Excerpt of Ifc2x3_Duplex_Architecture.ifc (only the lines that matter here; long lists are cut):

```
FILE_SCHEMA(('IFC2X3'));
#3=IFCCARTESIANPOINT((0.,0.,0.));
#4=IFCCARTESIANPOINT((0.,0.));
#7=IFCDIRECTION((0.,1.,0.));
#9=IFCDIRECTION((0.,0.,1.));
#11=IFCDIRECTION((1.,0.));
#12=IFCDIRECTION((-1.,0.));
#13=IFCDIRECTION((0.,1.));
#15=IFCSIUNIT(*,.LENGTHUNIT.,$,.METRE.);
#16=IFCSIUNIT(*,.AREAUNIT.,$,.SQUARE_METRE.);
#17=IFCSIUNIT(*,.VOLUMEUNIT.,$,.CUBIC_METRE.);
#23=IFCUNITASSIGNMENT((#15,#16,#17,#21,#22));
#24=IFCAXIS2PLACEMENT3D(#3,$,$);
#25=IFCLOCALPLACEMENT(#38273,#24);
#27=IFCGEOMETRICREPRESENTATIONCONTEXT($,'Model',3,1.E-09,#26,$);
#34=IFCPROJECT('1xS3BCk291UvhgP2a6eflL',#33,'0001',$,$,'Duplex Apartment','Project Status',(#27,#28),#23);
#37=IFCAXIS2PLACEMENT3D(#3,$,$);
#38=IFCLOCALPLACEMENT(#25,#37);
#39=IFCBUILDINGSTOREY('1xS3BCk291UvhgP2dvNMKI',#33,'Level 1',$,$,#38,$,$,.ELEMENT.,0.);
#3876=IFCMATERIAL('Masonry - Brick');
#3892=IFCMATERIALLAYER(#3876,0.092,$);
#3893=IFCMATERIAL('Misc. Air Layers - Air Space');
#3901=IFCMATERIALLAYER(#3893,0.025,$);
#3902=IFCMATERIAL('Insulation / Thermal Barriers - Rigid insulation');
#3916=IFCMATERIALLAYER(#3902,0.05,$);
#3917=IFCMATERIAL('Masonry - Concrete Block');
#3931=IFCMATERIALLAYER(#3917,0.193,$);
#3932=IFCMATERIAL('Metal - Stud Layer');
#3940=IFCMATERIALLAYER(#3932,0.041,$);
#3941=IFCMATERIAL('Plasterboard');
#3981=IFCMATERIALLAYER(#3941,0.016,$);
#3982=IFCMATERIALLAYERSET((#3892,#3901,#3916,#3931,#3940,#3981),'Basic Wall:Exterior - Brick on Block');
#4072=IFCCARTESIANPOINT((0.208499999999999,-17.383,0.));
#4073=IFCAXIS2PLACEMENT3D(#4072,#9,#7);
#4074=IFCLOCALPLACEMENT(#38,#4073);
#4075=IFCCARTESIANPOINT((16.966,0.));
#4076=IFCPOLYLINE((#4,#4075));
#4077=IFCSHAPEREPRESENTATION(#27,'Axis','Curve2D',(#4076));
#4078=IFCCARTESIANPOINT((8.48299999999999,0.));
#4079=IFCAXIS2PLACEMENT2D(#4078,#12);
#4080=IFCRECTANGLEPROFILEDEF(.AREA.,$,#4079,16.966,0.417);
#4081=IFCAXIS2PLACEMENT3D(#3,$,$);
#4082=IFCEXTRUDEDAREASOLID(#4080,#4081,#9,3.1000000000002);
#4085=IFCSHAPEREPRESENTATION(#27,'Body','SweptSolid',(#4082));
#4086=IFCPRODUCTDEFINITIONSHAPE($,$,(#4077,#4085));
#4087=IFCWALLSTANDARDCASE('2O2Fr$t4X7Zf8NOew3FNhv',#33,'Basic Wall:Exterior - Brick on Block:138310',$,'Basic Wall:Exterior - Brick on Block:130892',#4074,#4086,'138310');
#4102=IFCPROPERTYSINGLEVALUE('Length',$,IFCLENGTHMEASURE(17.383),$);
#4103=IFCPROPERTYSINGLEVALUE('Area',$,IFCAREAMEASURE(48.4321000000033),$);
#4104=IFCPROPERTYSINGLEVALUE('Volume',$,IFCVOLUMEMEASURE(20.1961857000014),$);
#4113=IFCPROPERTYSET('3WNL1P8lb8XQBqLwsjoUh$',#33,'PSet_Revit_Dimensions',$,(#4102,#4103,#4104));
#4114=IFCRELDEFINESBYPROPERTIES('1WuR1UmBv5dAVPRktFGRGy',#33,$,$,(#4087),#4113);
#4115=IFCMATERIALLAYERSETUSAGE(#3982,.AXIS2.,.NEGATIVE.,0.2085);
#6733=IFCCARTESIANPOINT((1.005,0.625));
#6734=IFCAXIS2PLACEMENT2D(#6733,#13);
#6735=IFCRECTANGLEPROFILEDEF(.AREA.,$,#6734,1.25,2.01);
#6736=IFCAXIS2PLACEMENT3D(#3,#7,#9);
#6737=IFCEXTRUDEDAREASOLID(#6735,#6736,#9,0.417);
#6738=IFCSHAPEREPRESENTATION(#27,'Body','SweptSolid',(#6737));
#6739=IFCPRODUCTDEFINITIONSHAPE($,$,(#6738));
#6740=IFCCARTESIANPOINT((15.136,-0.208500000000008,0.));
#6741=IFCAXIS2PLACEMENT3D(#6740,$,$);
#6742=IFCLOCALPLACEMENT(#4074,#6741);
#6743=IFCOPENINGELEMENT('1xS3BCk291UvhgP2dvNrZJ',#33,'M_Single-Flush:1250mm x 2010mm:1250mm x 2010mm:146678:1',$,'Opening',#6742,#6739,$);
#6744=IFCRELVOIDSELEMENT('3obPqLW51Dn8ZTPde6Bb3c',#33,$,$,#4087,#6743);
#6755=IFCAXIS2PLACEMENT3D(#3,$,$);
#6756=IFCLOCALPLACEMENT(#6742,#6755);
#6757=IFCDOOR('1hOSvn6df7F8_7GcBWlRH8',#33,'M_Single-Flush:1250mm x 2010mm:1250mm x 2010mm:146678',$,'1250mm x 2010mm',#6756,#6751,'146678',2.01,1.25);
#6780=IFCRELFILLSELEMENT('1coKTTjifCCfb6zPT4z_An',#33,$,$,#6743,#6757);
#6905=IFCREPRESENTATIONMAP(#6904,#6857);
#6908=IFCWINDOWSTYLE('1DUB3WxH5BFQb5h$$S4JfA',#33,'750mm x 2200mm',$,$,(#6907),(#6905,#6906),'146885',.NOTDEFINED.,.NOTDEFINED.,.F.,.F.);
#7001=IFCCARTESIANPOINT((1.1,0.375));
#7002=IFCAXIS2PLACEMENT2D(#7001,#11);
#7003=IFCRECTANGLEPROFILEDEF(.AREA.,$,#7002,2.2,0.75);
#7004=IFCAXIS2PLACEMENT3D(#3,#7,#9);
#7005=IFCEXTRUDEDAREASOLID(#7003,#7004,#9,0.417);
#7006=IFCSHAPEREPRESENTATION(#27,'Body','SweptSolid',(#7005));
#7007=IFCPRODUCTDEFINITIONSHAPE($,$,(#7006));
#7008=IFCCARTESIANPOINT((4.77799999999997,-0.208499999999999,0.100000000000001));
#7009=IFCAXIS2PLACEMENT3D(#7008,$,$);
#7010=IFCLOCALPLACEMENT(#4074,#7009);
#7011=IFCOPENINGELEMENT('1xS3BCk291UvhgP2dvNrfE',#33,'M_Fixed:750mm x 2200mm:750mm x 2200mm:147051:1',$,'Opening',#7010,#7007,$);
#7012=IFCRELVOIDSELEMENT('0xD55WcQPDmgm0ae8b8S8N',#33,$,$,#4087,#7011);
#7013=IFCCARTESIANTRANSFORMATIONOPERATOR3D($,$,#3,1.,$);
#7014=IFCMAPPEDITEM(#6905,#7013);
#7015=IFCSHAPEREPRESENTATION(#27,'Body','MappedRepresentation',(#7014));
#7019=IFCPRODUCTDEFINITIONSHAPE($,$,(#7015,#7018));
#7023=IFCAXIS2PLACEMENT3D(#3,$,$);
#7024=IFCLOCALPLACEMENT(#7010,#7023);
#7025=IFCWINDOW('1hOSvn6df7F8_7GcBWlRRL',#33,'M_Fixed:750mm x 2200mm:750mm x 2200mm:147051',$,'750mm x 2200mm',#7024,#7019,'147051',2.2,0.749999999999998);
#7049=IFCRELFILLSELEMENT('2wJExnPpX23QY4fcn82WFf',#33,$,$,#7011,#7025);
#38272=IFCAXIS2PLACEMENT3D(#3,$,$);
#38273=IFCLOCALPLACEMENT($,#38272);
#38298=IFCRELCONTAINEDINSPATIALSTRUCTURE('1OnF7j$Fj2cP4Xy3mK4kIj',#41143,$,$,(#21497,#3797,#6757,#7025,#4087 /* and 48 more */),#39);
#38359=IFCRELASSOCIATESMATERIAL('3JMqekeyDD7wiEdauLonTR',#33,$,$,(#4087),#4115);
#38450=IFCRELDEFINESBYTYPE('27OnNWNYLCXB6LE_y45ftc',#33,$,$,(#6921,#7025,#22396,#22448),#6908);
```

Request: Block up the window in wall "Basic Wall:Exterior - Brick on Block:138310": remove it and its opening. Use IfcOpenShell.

```python
import ifcopenshell
import ifcopenshell.api.feature
import ifcopenshell.api.pset
import ifcopenshell.api.root
import ifcopenshell.geom
import ifcopenshell.util.element
import ifcopenshell.util.shape
import ifcopenshell.util.unit

model = ifcopenshell.open("Ifc2x3_Duplex_Architecture.ifc")
area_scale = ifcopenshell.util.unit.calculate_unit_scale(model, "AREAUNIT")
volume_scale = ifcopenshell.util.unit.calculate_unit_scale(model, "VOLUMEUNIT")
settings = ifcopenshell.geom.settings()


def volume(element):
    """Net volume in cubic metres, openings subtracted."""
    shape = ifcopenshell.geom.create_shape(settings, element)
    return ifcopenshell.util.shape.get_volume(shape.geometry)


window = model.by_guid("1hOSvn6df7F8_7GcBWlRRL")
opening = window.FillsVoids[0].RelatingOpeningElement
wall = opening.VoidsElements[0].RelatingBuildingElement
before = volume(wall)

ifcopenshell.api.root.remove_product(model, product=window)
ifcopenshell.api.feature.remove_feature(model, feature=opening)

after = volume(wall)
thickness = 0.417  # wall thickness in metres

# Update the wall's stored quantities.
pset = model.by_id(ifcopenshell.util.element.get_pset(wall, "PSet_Revit_Dimensions", should_inherit=False)["id"])
ifcopenshell.api.pset.edit_pset(model, pset=pset, properties={
    "Area": model.create_entity("IfcAreaMeasure", after / thickness / area_scale),
    "Volume": model.create_entity("IfcVolumeMeasure", after / volume_scale),
})

print(f"wall volume {before:.3f} -> {after:.3f} m3")

model.write("Ifc2x3_Duplex_Architecture_updated.ifc")
```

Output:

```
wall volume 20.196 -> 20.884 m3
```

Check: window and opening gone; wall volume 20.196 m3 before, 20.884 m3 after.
